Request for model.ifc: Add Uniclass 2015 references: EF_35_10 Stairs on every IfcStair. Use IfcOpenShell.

First a look at what the model holds.

```python
import ifcopenshell

model = ifcopenshell.open("model.ifc")
print(model.schema)
print("classifications:", [c.Name for c in model.by_type("IfcClassification")])
for ifc_class in ("IfcDoor", "IfcRoof", "IfcStair", "IfcWall", "IfcWindow"):
    print(ifc_class, len(model.by_type(ifc_class)))
```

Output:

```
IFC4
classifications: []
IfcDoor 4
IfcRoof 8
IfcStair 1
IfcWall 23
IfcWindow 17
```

```python
import ifcopenshell
import ifcopenshell.api.classification

model = ifcopenshell.open("model.ifc")

system = ifcopenshell.api.classification.add_classification(model, classification="Uniclass 2015")

codes = {
    "IfcStair": ("EF_35_10", "Stairs"),
}
for ifc_class, (code, name) in codes.items():
    products = model.by_type(ifc_class)
    ifcopenshell.api.classification.add_reference(
        model, products=products, classification=system, identification=code, name=name
    )
    print(code, len(products))

model.write("model_updated.ifc")
```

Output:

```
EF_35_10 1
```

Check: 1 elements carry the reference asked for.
